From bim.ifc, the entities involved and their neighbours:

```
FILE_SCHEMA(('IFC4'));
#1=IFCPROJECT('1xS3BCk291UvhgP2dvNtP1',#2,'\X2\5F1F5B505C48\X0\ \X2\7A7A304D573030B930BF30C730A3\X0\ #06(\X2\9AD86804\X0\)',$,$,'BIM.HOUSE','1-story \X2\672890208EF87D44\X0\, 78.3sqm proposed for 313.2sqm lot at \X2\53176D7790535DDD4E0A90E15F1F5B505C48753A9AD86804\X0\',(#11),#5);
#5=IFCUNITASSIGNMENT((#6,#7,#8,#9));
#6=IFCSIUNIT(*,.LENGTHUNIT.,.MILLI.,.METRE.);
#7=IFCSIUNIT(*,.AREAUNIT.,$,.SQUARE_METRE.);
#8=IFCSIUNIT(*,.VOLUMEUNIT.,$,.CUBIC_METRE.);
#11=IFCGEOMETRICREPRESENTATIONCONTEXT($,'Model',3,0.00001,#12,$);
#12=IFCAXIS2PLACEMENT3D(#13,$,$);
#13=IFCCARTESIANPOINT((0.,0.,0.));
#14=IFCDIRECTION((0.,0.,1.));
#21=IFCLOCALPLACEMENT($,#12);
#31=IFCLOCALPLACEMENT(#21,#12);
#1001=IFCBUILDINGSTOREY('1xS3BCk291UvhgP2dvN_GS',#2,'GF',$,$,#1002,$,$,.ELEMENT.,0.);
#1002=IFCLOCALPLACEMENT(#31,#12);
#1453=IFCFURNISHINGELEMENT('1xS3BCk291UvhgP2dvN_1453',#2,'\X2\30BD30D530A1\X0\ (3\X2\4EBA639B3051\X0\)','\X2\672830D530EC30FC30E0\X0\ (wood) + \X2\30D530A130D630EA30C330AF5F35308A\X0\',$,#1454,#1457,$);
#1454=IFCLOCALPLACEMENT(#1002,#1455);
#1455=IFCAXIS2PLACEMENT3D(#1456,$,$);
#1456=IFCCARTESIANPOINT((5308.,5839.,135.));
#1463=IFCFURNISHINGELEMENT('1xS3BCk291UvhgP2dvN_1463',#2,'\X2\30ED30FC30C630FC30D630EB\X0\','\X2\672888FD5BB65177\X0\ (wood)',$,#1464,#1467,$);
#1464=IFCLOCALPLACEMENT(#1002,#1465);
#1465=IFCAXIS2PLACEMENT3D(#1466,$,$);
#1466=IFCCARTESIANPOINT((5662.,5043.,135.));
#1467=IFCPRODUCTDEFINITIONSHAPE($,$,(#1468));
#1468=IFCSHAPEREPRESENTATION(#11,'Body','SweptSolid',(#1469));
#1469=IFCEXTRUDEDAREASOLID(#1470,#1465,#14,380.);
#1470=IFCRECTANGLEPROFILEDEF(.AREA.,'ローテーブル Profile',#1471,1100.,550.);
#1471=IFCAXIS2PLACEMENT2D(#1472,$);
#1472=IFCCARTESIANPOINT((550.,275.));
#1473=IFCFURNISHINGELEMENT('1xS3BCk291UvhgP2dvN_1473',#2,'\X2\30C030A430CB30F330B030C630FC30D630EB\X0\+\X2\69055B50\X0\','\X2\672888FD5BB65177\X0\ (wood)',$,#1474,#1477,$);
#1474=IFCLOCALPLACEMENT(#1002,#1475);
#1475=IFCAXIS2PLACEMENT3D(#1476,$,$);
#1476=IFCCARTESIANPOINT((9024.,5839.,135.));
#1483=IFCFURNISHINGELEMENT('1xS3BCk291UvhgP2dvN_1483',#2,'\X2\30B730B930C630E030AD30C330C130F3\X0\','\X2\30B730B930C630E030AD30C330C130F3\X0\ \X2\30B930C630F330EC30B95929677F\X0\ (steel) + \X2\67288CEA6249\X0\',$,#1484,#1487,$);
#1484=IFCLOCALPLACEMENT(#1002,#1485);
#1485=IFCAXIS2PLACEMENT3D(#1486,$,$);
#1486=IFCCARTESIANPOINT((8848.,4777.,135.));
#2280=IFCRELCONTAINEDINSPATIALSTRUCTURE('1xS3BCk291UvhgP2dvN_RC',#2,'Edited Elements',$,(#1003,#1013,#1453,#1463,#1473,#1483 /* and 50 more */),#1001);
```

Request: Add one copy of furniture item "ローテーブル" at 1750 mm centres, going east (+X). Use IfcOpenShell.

```python
import numpy as np
import ifcopenshell
import ifcopenshell.api.geometry
import ifcopenshell.api.root
import ifcopenshell.util.element
import ifcopenshell.util.placement

model = ifcopenshell.open("bim.ifc")


def reuse_history(source, copy):
    """copy_class also copies each property set's owner history, people and application; keep the originals."""
    for rel in copy.IsDefinedBy:
        if rel.is_a("IfcRelDefinesByProperties") and (history := rel.RelatingPropertyDefinition.OwnerHistory):
            rel.RelatingPropertyDefinition.OwnerHistory = source.OwnerHistory
            ifcopenshell.util.element.remove_deep2(model, history)


source = model.by_guid("1xS3BCk291UvhgP2dvN_1463")
base = ifcopenshell.util.placement.get_local_placement(source.ObjectPlacement)
step = np.array([1.0, 0.0, 0.0]) * 1750.0

for i in range(1, 2):
    copy = ifcopenshell.api.root.copy_class(model, product=source)
    copy.Representation = ifcopenshell.util.element.copy_deep(
        model, source.Representation, exclude=["IfcGeometricRepresentationContext", "IfcRepresentationMap"]
    )
    reuse_history(source, copy)
    matrix = base.copy()
    matrix[:3, 3] += i * step
    print("added at", matrix[:3, 3].round(3) + 0.0)
    ifcopenshell.api.geometry.edit_object_placement(model, product=copy, matrix=matrix, is_si=False)

model.write("bim_rev.ifc")
```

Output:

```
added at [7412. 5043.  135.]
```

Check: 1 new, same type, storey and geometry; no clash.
